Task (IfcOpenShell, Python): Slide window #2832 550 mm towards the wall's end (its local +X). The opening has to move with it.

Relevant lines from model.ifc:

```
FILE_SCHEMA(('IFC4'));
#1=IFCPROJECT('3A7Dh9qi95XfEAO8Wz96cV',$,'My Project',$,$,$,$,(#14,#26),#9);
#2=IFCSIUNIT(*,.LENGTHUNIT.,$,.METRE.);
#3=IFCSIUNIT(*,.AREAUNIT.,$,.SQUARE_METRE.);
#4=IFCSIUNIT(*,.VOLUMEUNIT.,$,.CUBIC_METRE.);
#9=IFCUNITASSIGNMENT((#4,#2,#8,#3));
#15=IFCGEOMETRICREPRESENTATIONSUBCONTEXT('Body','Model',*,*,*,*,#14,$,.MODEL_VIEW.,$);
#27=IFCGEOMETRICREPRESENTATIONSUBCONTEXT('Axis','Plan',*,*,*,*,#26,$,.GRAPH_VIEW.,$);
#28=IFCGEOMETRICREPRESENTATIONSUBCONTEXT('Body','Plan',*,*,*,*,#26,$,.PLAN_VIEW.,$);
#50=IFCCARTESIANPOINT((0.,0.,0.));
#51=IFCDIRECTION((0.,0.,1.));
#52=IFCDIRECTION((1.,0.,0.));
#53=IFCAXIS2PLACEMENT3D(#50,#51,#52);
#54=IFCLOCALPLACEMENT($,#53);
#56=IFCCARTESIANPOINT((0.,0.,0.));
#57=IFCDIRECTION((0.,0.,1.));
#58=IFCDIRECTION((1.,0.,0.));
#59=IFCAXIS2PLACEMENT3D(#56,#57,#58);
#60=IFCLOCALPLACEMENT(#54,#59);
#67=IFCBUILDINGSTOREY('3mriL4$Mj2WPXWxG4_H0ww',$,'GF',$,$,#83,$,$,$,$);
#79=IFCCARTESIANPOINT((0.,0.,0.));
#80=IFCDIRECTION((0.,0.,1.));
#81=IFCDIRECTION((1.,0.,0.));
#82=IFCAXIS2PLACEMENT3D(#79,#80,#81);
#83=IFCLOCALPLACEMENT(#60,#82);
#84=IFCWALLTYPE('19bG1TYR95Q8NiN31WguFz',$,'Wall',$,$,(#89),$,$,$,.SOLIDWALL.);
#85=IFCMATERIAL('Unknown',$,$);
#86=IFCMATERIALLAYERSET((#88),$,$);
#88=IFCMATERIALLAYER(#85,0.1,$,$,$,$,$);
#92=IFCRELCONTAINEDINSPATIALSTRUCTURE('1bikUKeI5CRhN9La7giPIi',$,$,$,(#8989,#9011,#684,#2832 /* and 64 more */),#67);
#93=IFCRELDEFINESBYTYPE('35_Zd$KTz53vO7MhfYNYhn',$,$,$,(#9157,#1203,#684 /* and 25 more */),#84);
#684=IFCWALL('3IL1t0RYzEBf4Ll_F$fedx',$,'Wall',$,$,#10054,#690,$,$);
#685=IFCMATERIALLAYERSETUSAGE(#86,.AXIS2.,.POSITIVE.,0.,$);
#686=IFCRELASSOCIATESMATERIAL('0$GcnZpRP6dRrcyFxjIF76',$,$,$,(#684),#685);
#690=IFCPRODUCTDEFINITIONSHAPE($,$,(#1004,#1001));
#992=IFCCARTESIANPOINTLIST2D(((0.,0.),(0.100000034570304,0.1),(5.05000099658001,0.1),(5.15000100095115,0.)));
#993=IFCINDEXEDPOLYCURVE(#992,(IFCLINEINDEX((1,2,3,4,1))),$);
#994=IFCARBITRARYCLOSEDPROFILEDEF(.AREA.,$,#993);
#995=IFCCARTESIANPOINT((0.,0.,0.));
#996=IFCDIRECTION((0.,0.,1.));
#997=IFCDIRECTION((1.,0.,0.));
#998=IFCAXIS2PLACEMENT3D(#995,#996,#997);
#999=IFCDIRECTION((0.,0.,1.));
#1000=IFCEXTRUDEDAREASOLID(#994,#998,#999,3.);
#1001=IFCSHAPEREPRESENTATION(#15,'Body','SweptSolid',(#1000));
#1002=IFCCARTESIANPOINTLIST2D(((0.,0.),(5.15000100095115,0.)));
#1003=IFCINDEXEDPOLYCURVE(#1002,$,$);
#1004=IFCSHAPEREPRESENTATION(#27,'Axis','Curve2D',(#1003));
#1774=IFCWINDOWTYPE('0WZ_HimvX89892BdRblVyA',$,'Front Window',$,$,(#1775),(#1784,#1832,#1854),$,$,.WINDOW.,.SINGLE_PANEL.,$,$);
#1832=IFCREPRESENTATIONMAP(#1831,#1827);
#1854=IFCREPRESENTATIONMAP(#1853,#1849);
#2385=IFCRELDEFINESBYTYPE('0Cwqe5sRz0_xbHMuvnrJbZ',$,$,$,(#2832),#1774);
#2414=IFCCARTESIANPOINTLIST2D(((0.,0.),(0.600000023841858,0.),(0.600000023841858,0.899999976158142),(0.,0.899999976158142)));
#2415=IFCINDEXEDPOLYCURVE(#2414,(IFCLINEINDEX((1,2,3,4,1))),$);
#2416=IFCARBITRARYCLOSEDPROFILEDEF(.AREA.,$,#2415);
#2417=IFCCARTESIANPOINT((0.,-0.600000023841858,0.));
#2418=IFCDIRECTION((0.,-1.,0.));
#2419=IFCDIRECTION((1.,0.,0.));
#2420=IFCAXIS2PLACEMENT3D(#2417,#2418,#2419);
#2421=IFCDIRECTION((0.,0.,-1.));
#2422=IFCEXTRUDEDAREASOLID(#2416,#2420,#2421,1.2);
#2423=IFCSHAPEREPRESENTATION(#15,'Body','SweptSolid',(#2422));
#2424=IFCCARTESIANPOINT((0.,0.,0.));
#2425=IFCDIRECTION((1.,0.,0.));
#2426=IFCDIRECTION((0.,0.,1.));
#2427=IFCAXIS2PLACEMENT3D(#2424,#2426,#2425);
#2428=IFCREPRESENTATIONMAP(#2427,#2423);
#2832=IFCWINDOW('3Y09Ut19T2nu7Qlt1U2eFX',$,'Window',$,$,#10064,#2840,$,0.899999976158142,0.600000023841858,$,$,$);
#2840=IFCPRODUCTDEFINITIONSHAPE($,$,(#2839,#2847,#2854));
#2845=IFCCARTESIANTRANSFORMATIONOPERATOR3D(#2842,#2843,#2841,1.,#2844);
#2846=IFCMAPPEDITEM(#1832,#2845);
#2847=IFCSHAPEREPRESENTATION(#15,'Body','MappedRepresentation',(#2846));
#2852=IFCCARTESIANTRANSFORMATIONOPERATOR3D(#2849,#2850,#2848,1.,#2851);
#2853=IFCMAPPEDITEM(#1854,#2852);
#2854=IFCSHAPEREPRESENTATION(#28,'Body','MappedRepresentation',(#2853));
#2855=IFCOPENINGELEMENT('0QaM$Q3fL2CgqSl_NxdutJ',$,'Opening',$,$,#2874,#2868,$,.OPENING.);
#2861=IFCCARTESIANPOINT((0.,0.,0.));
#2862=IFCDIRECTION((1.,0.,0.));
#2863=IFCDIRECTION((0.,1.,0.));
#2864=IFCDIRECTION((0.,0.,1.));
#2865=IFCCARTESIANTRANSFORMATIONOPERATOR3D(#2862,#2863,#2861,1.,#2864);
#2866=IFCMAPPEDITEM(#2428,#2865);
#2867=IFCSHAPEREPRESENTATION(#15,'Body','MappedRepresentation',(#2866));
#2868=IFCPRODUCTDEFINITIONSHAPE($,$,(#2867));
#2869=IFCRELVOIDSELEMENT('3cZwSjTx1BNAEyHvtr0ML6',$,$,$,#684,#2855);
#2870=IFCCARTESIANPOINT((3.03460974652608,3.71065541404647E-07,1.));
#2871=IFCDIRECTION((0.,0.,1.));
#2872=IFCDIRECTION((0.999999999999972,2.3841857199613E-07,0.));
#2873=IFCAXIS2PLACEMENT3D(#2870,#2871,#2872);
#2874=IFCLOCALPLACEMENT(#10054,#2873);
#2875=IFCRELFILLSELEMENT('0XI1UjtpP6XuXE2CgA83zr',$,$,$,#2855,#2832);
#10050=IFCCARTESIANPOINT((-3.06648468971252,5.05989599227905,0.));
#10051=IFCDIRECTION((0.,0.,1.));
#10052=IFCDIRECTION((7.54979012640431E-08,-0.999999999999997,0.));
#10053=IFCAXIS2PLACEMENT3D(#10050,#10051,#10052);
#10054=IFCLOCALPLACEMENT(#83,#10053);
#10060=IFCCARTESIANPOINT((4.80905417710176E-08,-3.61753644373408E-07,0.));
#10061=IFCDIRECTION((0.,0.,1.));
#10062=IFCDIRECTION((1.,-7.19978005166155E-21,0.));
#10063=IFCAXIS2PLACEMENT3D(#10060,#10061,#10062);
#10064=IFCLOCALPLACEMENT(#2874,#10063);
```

```python
import ifcopenshell
import ifcopenshell.api.geometry
import ifcopenshell.util.placement
import ifcopenshell.util.unit

model = ifcopenshell.open("model.ifc")
unit_scale = ifcopenshell.util.unit.calculate_unit_scale(model)

window = model.by_guid("3Y09Ut19T2nu7Qlt1U2eFX")
opening = window.FillsVoids[0].RelatingOpeningElement
wall = opening.VoidsElements[0].RelatingBuildingElement

wall_matrix = ifcopenshell.util.placement.get_local_placement(wall.ObjectPlacement)
shift = wall_matrix[:3, 0] * 0.55 / unit_scale
before = ifcopenshell.util.placement.get_local_placement(window.ObjectPlacement)[:3, 3].copy()

# The window is placed relative to its opening, so it follows when the opening moves.
matrix = ifcopenshell.util.placement.get_local_placement(opening.ObjectPlacement)
matrix[:3, 3] += shift
ifcopenshell.api.geometry.edit_object_placement(
    model, product=opening, matrix=matrix, is_si=False, should_transform_children=True
)

after = ifcopenshell.util.placement.get_local_placement(window.ObjectPlacement)[:3, 3]
print("window moved by", (after - before).round(3) + 0.0)

model.write("model_v2.ifc")
```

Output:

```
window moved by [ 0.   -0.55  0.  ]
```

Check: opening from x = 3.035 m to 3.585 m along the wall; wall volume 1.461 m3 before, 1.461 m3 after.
